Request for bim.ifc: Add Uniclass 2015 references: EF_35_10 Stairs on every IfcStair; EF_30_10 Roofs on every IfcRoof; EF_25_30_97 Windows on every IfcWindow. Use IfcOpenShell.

First a look at what the model holds.

```python
import ifcopenshell

model = ifcopenshell.open("bim.ifc")
print(model.schema)
print("classifications:", [c.Name for c in model.by_type("IfcClassification")])
for ifc_class in ("IfcDoor", "IfcRoof", "IfcStair", "IfcWall", "IfcWindow"):
    print(ifc_class, len(model.by_type(ifc_class)))
```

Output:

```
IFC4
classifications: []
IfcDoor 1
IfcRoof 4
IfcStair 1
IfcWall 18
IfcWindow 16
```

```python
import ifcopenshell
import ifcopenshell.api.classification

model = ifcopenshell.open("bim.ifc")

system = ifcopenshell.api.classification.add_classification(model, classification="Uniclass 2015")

codes = {
    "IfcStair": ("EF_35_10", "Stairs"),
    "IfcRoof": ("EF_30_10", "Roofs"),
    "IfcWindow": ("EF_25_30_97", "Windows"),
}
for ifc_class, (code, name) in codes.items():
    products = model.by_type(ifc_class)
    ifcopenshell.api.classification.add_reference(
        model, products=products, classification=system, identification=code, name=name
    )
    print(code, len(products))

model.write("bim_edited.ifc")
```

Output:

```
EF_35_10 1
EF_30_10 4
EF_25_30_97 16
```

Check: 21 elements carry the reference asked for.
